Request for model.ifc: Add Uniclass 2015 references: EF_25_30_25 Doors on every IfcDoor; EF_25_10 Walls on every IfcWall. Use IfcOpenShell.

First a look at what the model holds.

```python
import ifcopenshell

model = ifcopenshell.open("model.ifc")
print(model.schema)
print("classifications:", [c.Name for c in model.by_type("IfcClassification")])
for ifc_class in ("IfcDoor", "IfcRoof", "IfcStair", "IfcWall", "IfcWindow"):
    print(ifc_class, len(model.by_type(ifc_class)))
```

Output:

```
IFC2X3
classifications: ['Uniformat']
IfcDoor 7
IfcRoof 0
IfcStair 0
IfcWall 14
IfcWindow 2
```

```python
import ifcopenshell
import ifcopenshell.api.classification

model = ifcopenshell.open("model.ifc")

# IFC2X3 requires Source and Edition and has no link from the project to the system.
system = model.create_entity("IfcClassification", Source="NBS", Edition="2015", Name="Uniclass 2015")

codes = {
    "IfcDoor": ("EF_25_30_25", "Doors"),
    "IfcWall": ("EF_25_10", "Walls"),
}
for ifc_class, (code, name) in codes.items():
    products = model.by_type(ifc_class)
    ifcopenshell.api.classification.add_reference(
        model, products=products, classification=system, identification=code, name=name
    )
    print(code, len(products))

model.write("model_rev.ifc")
```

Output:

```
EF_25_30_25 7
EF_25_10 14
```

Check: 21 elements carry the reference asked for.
